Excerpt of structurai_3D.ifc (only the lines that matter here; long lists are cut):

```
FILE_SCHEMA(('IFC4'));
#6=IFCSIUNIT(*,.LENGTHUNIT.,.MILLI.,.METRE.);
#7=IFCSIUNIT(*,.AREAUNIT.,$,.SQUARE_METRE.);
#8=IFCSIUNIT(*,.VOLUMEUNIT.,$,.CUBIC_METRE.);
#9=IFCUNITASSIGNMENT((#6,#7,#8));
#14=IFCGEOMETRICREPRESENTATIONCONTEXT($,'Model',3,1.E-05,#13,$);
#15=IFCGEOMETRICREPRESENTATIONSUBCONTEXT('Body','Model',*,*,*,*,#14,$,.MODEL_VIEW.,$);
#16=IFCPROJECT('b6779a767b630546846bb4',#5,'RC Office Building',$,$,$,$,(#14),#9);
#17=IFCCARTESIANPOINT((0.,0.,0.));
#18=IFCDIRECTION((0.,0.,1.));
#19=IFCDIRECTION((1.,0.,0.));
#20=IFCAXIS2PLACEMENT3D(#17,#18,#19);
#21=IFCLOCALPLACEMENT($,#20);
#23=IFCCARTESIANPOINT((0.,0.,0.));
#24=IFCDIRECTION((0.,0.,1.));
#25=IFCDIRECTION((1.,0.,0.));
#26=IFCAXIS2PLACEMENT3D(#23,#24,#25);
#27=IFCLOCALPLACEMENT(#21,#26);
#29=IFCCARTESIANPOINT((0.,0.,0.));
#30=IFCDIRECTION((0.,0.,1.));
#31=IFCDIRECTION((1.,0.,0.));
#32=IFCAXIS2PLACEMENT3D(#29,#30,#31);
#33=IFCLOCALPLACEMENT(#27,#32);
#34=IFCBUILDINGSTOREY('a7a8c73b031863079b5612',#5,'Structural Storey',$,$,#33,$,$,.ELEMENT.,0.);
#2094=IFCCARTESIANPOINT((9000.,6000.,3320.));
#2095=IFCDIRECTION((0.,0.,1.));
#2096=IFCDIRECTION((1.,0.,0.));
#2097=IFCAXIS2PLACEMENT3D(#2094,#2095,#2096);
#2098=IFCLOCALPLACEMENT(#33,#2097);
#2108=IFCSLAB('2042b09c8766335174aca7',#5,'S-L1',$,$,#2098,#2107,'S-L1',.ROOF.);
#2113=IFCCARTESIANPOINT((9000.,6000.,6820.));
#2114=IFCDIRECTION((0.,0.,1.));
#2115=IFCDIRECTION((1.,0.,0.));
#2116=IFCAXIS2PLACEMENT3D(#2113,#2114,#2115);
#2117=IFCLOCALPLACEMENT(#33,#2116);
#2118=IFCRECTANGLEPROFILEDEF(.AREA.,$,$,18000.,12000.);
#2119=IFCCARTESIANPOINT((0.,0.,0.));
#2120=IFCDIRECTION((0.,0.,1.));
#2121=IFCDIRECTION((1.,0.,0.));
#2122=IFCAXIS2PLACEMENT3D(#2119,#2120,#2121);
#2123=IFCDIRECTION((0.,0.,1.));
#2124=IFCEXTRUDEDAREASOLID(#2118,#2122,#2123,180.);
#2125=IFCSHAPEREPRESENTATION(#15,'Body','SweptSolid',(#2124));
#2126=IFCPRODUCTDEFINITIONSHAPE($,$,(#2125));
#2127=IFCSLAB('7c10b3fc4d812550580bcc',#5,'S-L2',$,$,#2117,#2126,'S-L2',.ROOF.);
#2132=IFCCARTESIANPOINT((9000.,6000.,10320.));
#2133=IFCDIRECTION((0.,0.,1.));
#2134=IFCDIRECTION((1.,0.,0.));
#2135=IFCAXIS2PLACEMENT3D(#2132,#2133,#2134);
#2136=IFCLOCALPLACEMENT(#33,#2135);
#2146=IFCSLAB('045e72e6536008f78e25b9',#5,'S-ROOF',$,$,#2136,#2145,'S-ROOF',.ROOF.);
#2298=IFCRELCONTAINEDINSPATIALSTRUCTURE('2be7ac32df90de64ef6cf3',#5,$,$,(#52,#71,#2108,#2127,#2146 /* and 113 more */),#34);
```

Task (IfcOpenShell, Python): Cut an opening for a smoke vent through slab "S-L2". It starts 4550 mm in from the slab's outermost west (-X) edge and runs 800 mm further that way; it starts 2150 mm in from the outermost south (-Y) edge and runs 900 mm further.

```python
import numpy as np
import ifcopenshell
import ifcopenshell.api.feature
import ifcopenshell.api.geometry
import ifcopenshell.api.root
import ifcopenshell.geom
import ifcopenshell.util.placement
import ifcopenshell.util.representation
import ifcopenshell.util.shape
import ifcopenshell.util.unit

model = ifcopenshell.open("structurai_3D.ifc")
unit_scale = ifcopenshell.util.unit.calculate_unit_scale(model)
settings = ifcopenshell.geom.settings()


def volume(element):
    """Net volume in cubic metres, openings subtracted."""
    shape = ifcopenshell.geom.create_shape(settings, element)
    return ifcopenshell.util.shape.get_volume(shape.geometry)


slab = model.by_guid("7c10b3fc4d812550580bcc")
before = volume(slab)

# Extent in the slab's own axes, in metres. The edges named are its -X and -Y sides.
slab_shape = ifcopenshell.geom.create_shape(settings, slab)
vertices = ifcopenshell.util.shape.get_vertices(slab_shape.geometry)
x_min, y_min, bottom = vertices.min(axis=0)
top = vertices[:, 2].max()

opening = ifcopenshell.api.root.create_entity(model, ifc_class="IfcOpeningElement", name="Smoke vent opening", predefined_type="OPENING")
context = ifcopenshell.util.representation.get_context(model, "Model", "Body", "MODEL_VIEW")
width, depth = 0.8, 0.9
outline = [(0.0, 0.0), (width, 0.0), (width, depth), (0.0, depth), (0.0, 0.0)]
# Overshoot both faces by 50 mm so the cut is clean.
shape = ifcopenshell.api.geometry.add_slab_representation(
    model, context=context, depth=top - bottom + 0.1, polyline=outline
)
ifcopenshell.api.geometry.assign_representation(model, product=opening, representation=shape)

matrix = ifcopenshell.util.placement.get_local_placement(slab.ObjectPlacement)
matrix[:, 3] = matrix @ np.append(np.array([x_min + 4.55, y_min + 2.15, bottom - 0.05]) / unit_scale, 1.0)
ifcopenshell.api.geometry.edit_object_placement(model, product=opening, matrix=matrix, is_si=False)
ifcopenshell.api.feature.add_feature(model, feature=opening, element=slab)

after = volume(slab)

print(f"slab volume {before:.3f} -> {after:.3f} m3")

model.write("structurai_3D_updated.ifc")
```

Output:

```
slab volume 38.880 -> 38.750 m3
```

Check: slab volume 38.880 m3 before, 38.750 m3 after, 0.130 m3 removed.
